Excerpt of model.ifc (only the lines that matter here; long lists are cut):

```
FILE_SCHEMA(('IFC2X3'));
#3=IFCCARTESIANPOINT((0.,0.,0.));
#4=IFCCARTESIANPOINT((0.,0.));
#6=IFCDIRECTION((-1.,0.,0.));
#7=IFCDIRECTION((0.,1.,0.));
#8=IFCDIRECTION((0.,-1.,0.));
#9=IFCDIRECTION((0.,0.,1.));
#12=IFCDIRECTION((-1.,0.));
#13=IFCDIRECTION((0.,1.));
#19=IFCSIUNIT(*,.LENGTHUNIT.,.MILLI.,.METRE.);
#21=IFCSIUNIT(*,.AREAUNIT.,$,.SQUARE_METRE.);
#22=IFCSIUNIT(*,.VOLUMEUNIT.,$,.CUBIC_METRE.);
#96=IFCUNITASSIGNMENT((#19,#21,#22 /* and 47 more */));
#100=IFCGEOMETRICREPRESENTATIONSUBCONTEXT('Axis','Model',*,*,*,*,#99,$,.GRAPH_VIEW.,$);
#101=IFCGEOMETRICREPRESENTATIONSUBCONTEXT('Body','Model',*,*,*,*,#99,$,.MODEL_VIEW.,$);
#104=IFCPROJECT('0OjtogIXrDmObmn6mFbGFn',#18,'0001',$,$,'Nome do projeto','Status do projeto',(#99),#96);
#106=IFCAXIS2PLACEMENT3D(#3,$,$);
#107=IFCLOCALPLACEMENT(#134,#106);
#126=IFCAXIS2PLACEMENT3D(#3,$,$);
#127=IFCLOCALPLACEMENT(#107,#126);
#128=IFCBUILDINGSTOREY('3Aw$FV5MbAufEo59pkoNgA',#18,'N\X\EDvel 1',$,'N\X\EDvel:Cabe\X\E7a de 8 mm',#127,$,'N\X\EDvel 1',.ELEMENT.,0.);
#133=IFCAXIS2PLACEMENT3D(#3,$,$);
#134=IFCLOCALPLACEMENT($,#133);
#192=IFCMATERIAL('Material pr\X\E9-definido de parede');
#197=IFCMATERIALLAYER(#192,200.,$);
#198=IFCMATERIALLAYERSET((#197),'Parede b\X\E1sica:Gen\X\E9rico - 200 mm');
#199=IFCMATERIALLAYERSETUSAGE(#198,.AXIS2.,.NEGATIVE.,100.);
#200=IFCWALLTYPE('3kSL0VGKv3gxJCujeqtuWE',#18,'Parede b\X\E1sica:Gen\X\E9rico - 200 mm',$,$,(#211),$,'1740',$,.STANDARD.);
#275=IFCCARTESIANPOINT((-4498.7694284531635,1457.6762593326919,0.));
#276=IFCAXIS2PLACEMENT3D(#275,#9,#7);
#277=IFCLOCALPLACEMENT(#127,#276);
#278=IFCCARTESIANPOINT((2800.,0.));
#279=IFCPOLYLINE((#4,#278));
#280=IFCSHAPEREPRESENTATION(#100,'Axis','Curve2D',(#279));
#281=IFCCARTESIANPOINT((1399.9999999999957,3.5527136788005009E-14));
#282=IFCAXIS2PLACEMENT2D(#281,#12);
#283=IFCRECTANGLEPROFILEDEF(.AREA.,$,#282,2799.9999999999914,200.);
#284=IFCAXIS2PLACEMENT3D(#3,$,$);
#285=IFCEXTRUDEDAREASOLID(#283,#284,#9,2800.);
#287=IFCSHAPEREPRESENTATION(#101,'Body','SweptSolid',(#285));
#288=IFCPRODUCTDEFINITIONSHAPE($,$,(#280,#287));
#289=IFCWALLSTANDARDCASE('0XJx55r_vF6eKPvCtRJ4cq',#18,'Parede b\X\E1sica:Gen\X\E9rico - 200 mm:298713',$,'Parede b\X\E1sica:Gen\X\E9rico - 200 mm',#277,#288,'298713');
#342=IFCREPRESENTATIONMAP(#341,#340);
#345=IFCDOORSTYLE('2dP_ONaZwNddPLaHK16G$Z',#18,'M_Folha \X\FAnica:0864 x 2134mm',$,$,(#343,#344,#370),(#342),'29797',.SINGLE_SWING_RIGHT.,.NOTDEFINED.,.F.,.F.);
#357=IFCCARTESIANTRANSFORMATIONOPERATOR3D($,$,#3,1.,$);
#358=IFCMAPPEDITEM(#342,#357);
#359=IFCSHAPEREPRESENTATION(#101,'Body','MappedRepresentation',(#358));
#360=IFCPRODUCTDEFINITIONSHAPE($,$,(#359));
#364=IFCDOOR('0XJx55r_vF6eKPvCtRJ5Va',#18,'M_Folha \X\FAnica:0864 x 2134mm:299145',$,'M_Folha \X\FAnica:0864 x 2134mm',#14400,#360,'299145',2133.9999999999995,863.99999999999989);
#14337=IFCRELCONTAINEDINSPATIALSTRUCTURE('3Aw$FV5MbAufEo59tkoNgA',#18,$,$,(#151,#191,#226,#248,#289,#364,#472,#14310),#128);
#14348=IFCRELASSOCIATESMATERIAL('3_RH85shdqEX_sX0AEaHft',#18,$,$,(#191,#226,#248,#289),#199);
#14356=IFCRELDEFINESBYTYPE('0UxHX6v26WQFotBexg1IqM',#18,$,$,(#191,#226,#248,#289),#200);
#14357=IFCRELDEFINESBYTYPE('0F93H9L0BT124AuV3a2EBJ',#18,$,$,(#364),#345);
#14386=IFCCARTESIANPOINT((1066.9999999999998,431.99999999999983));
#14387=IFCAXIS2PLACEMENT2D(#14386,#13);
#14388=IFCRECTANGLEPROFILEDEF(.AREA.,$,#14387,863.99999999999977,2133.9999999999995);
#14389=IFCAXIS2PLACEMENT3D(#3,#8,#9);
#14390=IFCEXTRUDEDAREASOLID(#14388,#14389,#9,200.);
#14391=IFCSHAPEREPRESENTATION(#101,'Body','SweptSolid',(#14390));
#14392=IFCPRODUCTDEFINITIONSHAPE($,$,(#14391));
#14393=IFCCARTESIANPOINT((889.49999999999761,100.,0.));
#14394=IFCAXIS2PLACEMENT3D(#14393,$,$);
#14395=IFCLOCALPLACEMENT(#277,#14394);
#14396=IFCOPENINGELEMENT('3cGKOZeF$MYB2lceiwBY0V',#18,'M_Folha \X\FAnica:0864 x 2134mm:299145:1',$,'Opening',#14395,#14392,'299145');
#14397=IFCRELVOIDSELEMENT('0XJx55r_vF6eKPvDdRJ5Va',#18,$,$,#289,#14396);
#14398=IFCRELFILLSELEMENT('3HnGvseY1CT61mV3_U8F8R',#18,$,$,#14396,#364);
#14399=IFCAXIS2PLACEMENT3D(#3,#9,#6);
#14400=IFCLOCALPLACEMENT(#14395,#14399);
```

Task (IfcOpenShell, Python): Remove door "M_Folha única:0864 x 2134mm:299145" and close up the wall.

```python
import ifcopenshell
import ifcopenshell.api.feature
import ifcopenshell.api.root
import ifcopenshell.geom
import ifcopenshell.util.shape

model = ifcopenshell.open("model.ifc")
settings = ifcopenshell.geom.settings()


def volume(element):
    """Net volume in cubic metres, openings subtracted."""
    shape = ifcopenshell.geom.create_shape(settings, element)
    return ifcopenshell.util.shape.get_volume(shape.geometry)


door = model.by_guid("0XJx55r_vF6eKPvCtRJ5Va")
opening = door.FillsVoids[0].RelatingOpeningElement
wall = opening.VoidsElements[0].RelatingBuildingElement
before = volume(wall)

ifcopenshell.api.root.remove_product(model, product=door)
ifcopenshell.api.feature.remove_feature(model, feature=opening)

after = volume(wall)

print(f"wall volume {before:.3f} -> {after:.3f} m3")

model.write("model_rev.ifc")
```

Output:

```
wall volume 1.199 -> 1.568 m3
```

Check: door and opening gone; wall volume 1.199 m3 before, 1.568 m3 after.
